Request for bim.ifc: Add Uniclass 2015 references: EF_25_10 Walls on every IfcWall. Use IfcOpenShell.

First a look at what the model holds.

```python
import ifcopenshell

model = ifcopenshell.open("bim.ifc")
print(model.schema)
print("classifications:", [c.Name for c in model.by_type("IfcClassification")])
for ifc_class in ("IfcDoor", "IfcRoof", "IfcStair", "IfcWall", "IfcWindow"):
    print(ifc_class, len(model.by_type(ifc_class)))
```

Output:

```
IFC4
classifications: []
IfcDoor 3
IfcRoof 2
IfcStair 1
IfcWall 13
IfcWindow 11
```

```python
import ifcopenshell
import ifcopenshell.api.classification

model = ifcopenshell.open("bim.ifc")

system = ifcopenshell.api.classification.add_classification(model, classification="Uniclass 2015")

codes = {
    "IfcWall": ("EF_25_10", "Walls"),
}
for ifc_class, (code, name) in codes.items():
    products = model.by_type(ifc_class)
    ifcopenshell.api.classification.add_reference(
        model, products=products, classification=system, identification=code, name=name
    )
    print(code, len(products))

model.write("bim_rev.ifc")
```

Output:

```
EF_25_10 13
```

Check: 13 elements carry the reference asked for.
